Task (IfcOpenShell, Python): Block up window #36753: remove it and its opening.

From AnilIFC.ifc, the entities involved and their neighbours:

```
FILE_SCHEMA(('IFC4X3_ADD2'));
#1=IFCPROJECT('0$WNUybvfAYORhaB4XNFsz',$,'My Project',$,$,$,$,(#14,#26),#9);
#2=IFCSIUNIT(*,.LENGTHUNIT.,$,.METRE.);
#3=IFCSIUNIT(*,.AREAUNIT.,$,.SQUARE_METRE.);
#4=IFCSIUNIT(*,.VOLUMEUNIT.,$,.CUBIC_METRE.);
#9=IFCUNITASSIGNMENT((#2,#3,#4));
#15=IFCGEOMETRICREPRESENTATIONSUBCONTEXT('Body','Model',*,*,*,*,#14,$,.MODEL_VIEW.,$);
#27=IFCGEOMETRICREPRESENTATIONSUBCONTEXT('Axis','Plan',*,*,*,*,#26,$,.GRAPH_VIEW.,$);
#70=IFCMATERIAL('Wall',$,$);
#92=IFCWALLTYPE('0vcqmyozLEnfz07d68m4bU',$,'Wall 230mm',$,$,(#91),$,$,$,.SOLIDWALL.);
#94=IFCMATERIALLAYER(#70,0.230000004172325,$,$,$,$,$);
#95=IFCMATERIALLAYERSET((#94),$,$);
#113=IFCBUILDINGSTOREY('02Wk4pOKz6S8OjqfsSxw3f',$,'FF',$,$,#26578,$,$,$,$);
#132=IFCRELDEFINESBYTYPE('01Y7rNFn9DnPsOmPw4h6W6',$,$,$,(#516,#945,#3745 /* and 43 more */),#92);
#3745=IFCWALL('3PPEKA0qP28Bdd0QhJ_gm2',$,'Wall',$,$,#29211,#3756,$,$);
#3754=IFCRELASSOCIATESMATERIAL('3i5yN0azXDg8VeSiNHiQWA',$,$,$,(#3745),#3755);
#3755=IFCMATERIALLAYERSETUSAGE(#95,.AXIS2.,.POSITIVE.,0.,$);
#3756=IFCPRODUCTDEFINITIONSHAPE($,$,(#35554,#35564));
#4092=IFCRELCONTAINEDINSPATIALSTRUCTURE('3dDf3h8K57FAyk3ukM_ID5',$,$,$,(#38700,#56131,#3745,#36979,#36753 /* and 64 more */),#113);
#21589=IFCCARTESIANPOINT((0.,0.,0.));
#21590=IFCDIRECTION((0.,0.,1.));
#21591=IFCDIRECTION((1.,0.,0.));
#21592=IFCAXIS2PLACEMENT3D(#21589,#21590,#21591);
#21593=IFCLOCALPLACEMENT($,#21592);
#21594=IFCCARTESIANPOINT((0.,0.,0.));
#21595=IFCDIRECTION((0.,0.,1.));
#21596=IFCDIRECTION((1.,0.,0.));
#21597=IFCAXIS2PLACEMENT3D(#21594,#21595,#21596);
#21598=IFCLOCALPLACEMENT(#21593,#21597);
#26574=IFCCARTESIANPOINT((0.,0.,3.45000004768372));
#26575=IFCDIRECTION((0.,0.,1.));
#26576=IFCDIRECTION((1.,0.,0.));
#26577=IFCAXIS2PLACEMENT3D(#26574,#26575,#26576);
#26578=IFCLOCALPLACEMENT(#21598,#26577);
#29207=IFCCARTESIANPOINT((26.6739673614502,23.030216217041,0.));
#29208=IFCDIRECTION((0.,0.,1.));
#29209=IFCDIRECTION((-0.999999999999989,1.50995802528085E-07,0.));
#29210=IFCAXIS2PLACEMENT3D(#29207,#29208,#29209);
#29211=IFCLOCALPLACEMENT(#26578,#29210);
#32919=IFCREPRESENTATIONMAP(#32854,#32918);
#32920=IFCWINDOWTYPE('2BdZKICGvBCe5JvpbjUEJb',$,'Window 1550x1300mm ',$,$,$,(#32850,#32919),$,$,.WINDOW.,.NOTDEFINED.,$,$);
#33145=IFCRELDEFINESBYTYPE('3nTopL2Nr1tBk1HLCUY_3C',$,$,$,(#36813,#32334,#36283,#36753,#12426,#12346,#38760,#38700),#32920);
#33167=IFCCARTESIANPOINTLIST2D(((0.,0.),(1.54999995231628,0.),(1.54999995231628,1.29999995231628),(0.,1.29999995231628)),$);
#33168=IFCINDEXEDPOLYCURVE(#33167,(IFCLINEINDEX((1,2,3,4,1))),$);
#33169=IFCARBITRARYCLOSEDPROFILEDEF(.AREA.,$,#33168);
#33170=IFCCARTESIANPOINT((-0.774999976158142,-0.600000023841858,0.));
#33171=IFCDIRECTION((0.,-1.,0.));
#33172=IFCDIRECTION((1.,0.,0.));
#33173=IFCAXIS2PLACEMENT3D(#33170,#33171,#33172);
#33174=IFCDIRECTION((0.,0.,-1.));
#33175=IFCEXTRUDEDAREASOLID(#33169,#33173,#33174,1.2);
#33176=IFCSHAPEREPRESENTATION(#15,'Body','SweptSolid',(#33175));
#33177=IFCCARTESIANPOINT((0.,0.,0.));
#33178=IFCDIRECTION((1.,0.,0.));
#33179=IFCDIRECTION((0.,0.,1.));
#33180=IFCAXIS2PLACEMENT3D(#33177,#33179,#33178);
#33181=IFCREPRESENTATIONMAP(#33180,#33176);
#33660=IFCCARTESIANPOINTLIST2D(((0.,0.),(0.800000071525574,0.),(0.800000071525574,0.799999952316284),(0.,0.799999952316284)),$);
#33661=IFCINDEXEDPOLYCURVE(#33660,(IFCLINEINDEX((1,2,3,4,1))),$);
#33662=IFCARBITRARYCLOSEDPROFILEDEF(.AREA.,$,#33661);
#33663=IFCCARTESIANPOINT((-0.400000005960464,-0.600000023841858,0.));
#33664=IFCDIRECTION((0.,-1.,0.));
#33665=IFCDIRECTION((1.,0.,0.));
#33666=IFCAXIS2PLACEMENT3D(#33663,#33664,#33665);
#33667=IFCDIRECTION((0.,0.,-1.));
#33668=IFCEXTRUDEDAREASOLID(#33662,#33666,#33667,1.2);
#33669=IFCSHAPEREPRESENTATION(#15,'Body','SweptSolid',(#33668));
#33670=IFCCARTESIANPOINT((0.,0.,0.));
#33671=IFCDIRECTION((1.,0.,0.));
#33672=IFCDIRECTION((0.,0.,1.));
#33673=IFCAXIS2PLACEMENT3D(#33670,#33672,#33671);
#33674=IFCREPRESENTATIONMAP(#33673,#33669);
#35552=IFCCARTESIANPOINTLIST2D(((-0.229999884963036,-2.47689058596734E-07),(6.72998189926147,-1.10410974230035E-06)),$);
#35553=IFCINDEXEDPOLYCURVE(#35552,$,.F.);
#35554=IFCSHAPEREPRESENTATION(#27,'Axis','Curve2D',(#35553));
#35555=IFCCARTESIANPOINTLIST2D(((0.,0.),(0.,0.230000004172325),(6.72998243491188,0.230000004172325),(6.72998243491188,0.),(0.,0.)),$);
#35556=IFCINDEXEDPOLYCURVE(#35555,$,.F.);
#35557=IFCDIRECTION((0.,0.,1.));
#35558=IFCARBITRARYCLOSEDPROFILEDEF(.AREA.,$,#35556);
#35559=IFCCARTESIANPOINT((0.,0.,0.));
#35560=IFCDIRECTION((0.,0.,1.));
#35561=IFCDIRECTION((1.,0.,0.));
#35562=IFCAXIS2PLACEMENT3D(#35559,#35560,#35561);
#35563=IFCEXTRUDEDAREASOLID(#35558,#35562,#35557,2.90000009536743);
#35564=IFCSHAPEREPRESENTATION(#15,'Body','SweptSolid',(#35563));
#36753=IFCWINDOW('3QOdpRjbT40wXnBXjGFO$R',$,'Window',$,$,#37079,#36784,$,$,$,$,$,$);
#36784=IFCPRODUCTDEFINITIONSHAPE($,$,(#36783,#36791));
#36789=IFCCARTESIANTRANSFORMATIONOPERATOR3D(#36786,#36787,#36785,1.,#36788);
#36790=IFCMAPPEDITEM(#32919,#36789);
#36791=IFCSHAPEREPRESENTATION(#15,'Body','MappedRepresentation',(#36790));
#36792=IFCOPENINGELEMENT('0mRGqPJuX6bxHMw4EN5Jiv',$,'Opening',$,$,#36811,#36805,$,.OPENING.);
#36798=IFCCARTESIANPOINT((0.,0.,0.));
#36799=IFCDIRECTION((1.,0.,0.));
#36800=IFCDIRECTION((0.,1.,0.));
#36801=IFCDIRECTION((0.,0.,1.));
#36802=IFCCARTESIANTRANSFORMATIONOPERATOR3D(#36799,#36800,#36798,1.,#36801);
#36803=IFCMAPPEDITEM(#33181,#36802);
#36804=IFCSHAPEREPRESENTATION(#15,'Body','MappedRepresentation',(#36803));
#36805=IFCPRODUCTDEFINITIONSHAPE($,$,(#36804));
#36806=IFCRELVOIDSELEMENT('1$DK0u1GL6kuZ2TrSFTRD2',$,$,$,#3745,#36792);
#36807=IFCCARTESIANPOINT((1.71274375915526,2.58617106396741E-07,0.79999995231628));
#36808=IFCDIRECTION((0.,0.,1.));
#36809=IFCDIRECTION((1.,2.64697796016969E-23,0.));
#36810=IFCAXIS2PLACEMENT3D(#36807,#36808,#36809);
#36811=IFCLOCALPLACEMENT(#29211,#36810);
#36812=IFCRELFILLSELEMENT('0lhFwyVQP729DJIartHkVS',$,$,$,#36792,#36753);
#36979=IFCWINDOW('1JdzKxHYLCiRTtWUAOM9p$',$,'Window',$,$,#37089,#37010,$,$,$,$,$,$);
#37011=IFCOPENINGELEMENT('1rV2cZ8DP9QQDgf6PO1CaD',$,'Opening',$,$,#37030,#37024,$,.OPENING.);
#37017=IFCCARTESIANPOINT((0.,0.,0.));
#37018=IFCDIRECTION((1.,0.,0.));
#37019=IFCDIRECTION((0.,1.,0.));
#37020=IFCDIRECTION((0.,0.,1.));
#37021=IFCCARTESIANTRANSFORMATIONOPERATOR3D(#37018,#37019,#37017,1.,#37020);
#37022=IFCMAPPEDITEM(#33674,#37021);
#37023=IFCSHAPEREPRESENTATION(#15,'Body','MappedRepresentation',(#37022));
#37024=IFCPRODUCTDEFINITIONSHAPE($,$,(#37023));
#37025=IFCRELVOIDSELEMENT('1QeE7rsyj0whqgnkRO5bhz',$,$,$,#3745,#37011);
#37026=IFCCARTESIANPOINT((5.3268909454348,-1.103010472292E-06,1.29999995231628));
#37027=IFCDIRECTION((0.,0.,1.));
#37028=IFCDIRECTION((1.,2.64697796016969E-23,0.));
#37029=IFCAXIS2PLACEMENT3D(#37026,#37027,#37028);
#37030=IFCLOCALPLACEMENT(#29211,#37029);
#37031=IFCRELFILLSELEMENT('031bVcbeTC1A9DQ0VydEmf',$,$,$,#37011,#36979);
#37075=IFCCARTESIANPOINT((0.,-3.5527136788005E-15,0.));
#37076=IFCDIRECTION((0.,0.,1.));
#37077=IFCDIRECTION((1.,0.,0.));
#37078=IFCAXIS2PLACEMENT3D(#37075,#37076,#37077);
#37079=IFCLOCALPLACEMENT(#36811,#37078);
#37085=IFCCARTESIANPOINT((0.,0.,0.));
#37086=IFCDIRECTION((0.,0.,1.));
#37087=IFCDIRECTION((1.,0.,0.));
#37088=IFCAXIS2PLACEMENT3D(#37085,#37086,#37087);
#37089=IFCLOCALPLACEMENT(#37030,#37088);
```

```python
import ifcopenshell
import ifcopenshell.api.feature
import ifcopenshell.api.root
import ifcopenshell.geom
import ifcopenshell.util.shape

model = ifcopenshell.open("AnilIFC.ifc")
settings = ifcopenshell.geom.settings()


def volume(element):
    """Net volume in cubic metres, openings subtracted."""
    shape = ifcopenshell.geom.create_shape(settings, element)
    return ifcopenshell.util.shape.get_volume(shape.geometry)


window = model.by_guid("3QOdpRjbT40wXnBXjGFO$R")
opening = window.FillsVoids[0].RelatingOpeningElement
wall = opening.VoidsElements[0].RelatingBuildingElement
before = volume(wall)

ifcopenshell.api.root.remove_product(model, product=window)
ifcopenshell.api.feature.remove_feature(model, feature=opening)

after = volume(wall)

print(f"wall volume {before:.3f} -> {after:.3f} m3")

model.write("AnilIFC-out.ifc")
```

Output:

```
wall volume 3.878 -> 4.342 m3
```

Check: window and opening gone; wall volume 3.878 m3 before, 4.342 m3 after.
